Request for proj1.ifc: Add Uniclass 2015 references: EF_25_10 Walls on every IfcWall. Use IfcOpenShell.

First a look at what the model holds.

```python
import ifcopenshell

model = ifcopenshell.open("proj1.ifc")
print(model.schema)
print("classifications:", [c.Name for c in model.by_type("IfcClassification")])
for ifc_class in ("IfcDoor", "IfcRoof", "IfcStair", "IfcWall", "IfcWindow"):
    print(ifc_class, len(model.by_type(ifc_class)))
```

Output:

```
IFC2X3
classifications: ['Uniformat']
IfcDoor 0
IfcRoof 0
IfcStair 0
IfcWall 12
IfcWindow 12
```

```python
import ifcopenshell
import ifcopenshell.api.classification

model = ifcopenshell.open("proj1.ifc")

# IFC2X3 requires Source and Edition and has no link from the project to the system.
system = model.create_entity("IfcClassification", Source="NBS", Edition="2015", Name="Uniclass 2015")

codes = {
    "IfcWall": ("EF_25_10", "Walls"),
}
for ifc_class, (code, name) in codes.items():
    products = model.by_type(ifc_class)
    ifcopenshell.api.classification.add_reference(
        model, products=products, classification=system, identification=code, name=name
    )
    print(code, len(products))

model.write("proj1_updated.ifc")
```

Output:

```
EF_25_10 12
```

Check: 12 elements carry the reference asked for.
